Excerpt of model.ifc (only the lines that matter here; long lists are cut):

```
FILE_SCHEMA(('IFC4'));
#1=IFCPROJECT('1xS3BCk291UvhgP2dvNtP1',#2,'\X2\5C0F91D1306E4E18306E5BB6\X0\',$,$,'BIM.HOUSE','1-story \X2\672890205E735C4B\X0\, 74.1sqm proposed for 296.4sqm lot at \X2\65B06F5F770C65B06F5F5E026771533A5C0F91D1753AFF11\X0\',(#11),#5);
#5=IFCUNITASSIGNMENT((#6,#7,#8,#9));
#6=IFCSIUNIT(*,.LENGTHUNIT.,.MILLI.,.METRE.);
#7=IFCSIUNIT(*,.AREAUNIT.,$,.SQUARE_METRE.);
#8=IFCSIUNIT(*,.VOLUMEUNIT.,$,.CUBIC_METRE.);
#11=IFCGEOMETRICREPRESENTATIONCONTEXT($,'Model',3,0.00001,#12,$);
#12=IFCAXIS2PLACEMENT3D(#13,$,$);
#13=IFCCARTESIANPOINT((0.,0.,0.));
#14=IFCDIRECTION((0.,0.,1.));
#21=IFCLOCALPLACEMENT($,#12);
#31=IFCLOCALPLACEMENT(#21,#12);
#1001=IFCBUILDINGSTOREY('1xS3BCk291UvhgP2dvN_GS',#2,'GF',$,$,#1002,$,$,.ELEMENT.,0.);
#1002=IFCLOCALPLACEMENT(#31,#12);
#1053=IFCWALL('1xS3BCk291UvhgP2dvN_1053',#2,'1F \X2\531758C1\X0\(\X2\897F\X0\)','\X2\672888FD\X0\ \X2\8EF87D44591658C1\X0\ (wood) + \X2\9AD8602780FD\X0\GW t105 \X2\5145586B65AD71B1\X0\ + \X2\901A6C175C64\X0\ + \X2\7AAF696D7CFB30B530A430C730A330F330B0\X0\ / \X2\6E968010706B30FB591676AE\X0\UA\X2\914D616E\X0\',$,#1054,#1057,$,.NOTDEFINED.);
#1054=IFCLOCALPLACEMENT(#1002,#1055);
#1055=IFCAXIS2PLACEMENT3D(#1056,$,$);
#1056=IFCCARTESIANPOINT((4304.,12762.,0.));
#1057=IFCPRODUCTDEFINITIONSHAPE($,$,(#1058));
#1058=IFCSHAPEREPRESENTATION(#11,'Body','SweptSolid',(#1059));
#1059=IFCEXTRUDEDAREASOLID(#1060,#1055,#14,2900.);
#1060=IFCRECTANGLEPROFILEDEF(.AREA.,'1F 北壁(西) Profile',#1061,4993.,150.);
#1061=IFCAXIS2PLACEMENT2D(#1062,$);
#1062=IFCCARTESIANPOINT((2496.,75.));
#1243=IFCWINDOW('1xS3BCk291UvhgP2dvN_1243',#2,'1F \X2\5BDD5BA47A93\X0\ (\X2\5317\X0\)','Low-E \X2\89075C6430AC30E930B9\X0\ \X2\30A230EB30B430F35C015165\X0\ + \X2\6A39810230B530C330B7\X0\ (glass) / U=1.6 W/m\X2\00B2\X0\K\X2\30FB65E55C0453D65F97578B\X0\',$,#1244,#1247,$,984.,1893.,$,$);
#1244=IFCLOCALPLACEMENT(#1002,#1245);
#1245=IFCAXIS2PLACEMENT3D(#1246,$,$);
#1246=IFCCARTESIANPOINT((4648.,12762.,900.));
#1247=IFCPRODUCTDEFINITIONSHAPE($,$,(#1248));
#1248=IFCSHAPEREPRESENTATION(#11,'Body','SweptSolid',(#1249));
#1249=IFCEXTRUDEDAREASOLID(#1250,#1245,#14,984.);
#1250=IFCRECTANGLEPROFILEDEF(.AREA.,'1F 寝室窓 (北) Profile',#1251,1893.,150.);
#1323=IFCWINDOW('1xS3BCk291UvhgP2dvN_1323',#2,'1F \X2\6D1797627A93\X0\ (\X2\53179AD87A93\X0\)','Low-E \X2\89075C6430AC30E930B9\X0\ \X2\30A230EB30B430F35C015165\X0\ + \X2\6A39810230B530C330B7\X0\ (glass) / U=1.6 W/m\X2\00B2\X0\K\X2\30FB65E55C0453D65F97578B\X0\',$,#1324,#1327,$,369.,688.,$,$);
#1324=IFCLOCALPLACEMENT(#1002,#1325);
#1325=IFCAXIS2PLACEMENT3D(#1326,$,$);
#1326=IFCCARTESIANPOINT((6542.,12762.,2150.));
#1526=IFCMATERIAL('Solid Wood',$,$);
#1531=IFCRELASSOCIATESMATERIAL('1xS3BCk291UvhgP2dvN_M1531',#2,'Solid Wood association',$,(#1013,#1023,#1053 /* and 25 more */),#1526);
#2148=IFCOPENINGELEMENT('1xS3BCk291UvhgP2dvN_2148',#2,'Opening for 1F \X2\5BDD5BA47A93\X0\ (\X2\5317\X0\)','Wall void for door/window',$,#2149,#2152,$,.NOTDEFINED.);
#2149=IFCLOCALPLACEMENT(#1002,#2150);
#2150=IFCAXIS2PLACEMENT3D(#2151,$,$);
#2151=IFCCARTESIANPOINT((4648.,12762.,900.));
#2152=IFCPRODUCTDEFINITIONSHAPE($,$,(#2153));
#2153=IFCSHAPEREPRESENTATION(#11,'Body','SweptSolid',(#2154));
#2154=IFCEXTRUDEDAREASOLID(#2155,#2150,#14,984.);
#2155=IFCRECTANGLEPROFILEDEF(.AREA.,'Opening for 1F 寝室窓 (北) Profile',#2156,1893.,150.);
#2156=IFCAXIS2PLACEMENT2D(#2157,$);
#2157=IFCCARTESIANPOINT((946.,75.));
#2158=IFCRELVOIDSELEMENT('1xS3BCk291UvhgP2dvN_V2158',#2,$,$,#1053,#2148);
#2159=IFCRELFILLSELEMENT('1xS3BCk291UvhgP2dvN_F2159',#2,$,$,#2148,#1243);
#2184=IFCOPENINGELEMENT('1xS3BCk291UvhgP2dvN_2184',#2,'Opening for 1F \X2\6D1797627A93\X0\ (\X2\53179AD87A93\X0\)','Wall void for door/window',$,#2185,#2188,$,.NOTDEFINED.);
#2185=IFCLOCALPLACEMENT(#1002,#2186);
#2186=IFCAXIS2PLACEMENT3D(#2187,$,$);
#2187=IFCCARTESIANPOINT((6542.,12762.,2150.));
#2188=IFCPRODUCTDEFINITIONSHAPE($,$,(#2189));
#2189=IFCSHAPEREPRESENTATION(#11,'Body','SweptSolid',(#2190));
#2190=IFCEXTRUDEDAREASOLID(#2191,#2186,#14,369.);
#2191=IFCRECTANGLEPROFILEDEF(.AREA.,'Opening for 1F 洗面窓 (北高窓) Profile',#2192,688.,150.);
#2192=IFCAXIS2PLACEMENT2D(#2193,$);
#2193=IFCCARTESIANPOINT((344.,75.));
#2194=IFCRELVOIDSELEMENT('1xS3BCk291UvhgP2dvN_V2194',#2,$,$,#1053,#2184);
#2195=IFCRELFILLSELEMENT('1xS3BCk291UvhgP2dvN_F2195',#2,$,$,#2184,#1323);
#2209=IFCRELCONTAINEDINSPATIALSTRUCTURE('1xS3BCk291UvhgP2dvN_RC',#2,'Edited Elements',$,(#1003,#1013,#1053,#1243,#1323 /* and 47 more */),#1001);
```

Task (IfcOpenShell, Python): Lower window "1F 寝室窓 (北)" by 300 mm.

```python
import numpy as np
import ifcopenshell
import ifcopenshell.api.geometry
import ifcopenshell.util.placement
import ifcopenshell.util.unit

model = ifcopenshell.open("model.ifc")
unit_scale = ifcopenshell.util.unit.calculate_unit_scale(model)

window = model.by_guid("1xS3BCk291UvhgP2dvN_1243")
opening = window.FillsVoids[0].RelatingOpeningElement
dz = -300.0

shift = np.array([0.0, 0.0, dz])
# The window is not placed relative to its opening, so move both.
for product in (opening, window):
    matrix = ifcopenshell.util.placement.get_local_placement(product.ObjectPlacement)
    matrix[:3, 3] += shift
    ifcopenshell.api.geometry.edit_object_placement(model, product=product, matrix=matrix, is_si=False)

print(f"moved by {dz * unit_scale:+.3f} m")

model.write("model_updated.ifc")
```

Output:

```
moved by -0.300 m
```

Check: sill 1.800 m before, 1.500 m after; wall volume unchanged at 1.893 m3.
